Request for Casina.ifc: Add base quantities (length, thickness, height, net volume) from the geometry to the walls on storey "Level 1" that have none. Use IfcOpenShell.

First a look at what the model holds.

```python
import ifcopenshell
import ifcopenshell.util.element
import ifcopenshell.util.unit

model = ifcopenshell.open("Casina.ifc")
print(model.schema)
for unit_type in ("LENGTHUNIT", "AREAUNIT", "VOLUMEUNIT"):
    print(unit_type, ifcopenshell.util.unit.calculate_unit_scale(model, unit_type))
storey = next(s for s in model.by_type("IfcBuildingStorey") if s.Name == "Level 1")
walls = [e for e in ifcopenshell.util.element.get_decomposition(storey) if e.is_a("IfcWall")]
for e in sorted(walls, key=lambda e: e.id()):
    print(e.id(), e.is_a(), e.Name, list(ifcopenshell.util.element.get_psets(e, qtos_only=True)), sep=" | ")
```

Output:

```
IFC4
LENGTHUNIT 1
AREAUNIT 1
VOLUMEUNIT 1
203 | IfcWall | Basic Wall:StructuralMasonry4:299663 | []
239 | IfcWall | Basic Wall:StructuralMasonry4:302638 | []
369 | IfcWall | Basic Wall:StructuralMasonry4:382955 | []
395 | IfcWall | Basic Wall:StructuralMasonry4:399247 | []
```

```python
import ifcopenshell
import ifcopenshell.api.pset
import ifcopenshell.geom
import ifcopenshell.util.element
import ifcopenshell.util.shape
import ifcopenshell.util.unit

model = ifcopenshell.open("Casina.ifc")
unit_scale = ifcopenshell.util.unit.calculate_unit_scale(model)
volume_scale = ifcopenshell.util.unit.calculate_unit_scale(model, "VOLUMEUNIT")
settings = ifcopenshell.geom.settings()

storey = next(s for s in model.by_type("IfcBuildingStorey") if s.Name == "Level 1")
walls = [e for e in ifcopenshell.util.element.get_decomposition(storey) if e.is_a("IfcWall")]

for e in sorted(walls, key=lambda e: e.id()):
    if ifcopenshell.util.element.get_psets(e, qtos_only=True, should_inherit=False):
        continue
    # Geometry comes back in metres, in the element's own axes.
    shape = ifcopenshell.geom.create_shape(settings, e)
    values = {
        "Length": ifcopenshell.util.shape.get_x(shape.geometry) / unit_scale,
        "Width": ifcopenshell.util.shape.get_y(shape.geometry) / unit_scale,
        "Height": ifcopenshell.util.shape.get_z(shape.geometry) / unit_scale,
        "NetVolume": ifcopenshell.util.shape.get_volume(shape.geometry) / volume_scale,
    }
    qto = ifcopenshell.api.pset.add_qto(model, product=e, name="Qto_WallBaseQuantities")
    ifcopenshell.api.pset.edit_qto(model, qto=qto, properties=values)
    print(e.id(), {k: round(v, 3) for k, v in values.items()})

model.write("Casina-out.ifc")
```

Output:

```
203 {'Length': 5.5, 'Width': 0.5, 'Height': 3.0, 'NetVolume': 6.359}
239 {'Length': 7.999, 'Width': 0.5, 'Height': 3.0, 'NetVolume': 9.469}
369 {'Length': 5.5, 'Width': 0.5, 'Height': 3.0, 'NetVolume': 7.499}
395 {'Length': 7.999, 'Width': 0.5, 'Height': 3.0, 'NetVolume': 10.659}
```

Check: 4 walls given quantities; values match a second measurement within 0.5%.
